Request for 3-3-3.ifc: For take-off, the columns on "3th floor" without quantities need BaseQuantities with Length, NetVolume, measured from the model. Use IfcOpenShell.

First a look at what the model holds.

```python
import ifcopenshell
import ifcopenshell.util.element
import ifcopenshell.util.unit

model = ifcopenshell.open("3-3-3.ifc")
print(model.schema)
for unit_type in ("LENGTHUNIT", "AREAUNIT", "VOLUMEUNIT"):
    print(unit_type, ifcopenshell.util.unit.calculate_unit_scale(model, unit_type))
storey = next(s for s in model.by_type("IfcBuildingStorey") if s.Name == "3th floor")
columns = [e for e in ifcopenshell.util.element.get_decomposition(storey) if e.is_a("IfcColumn")]
for e in sorted(columns, key=lambda e: e.id()):
    print(e.id(), e.is_a(), e.Name, list(ifcopenshell.util.element.get_psets(e, qtos_only=True)), sep=" | ")
```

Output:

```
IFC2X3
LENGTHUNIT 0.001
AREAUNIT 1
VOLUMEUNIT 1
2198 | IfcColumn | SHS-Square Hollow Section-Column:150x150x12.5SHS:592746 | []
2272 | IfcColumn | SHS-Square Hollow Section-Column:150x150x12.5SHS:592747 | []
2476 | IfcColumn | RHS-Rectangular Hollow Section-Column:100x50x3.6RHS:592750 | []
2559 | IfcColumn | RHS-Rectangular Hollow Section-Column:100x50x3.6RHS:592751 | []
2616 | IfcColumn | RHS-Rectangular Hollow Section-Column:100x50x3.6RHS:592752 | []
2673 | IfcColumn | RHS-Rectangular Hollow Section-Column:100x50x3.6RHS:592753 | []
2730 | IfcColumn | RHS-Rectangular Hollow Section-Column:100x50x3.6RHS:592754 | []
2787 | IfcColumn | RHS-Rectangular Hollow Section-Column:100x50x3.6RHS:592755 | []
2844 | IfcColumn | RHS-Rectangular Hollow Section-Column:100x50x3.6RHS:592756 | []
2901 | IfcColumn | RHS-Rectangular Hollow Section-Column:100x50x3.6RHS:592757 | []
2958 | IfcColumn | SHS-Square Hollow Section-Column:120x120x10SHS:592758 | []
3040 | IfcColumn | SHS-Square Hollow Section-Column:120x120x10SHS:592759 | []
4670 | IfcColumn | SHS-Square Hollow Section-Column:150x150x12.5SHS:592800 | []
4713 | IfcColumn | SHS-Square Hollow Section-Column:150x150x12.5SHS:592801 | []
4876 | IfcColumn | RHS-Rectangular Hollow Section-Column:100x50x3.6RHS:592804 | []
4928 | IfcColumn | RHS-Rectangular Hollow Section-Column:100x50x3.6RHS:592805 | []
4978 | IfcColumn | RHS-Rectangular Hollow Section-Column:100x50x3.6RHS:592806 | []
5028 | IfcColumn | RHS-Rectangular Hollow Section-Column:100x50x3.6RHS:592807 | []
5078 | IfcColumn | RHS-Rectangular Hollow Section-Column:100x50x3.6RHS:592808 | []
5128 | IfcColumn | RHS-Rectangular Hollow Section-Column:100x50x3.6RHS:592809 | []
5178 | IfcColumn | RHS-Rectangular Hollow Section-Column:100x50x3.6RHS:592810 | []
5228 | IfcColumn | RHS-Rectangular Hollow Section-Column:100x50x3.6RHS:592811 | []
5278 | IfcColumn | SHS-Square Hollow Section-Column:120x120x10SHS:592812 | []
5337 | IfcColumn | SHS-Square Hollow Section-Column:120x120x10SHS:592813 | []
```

```python
import ifcopenshell
import ifcopenshell.api.pset
import ifcopenshell.geom
import ifcopenshell.util.element
import ifcopenshell.util.shape
import ifcopenshell.util.unit

model = ifcopenshell.open("3-3-3.ifc")
unit_scale = ifcopenshell.util.unit.calculate_unit_scale(model)
volume_scale = ifcopenshell.util.unit.calculate_unit_scale(model, "VOLUMEUNIT")
settings = ifcopenshell.geom.settings()

storey = next(s for s in model.by_type("IfcBuildingStorey") if s.Name == "3th floor")
columns = [e for e in ifcopenshell.util.element.get_decomposition(storey) if e.is_a("IfcColumn")]

for e in sorted(columns, key=lambda e: e.id()):
    if ifcopenshell.util.element.get_psets(e, qtos_only=True, should_inherit=False):
        continue
    # Geometry comes back in metres, in the element's own axes.
    shape = ifcopenshell.geom.create_shape(settings, e)
    values = {
        "Length": ifcopenshell.util.shape.get_z(shape.geometry) / unit_scale,
        "NetVolume": ifcopenshell.util.shape.get_volume(shape.geometry) / volume_scale,
    }
    qto = ifcopenshell.api.pset.add_qto(model, product=e, name="BaseQuantities")
    ifcopenshell.api.pset.edit_qto(model, qto=qto, properties=values)
    print(e.id(), {k: round(v, 3) for k, v in values.items()})

model.write("3-3-3_v2.ifc")
```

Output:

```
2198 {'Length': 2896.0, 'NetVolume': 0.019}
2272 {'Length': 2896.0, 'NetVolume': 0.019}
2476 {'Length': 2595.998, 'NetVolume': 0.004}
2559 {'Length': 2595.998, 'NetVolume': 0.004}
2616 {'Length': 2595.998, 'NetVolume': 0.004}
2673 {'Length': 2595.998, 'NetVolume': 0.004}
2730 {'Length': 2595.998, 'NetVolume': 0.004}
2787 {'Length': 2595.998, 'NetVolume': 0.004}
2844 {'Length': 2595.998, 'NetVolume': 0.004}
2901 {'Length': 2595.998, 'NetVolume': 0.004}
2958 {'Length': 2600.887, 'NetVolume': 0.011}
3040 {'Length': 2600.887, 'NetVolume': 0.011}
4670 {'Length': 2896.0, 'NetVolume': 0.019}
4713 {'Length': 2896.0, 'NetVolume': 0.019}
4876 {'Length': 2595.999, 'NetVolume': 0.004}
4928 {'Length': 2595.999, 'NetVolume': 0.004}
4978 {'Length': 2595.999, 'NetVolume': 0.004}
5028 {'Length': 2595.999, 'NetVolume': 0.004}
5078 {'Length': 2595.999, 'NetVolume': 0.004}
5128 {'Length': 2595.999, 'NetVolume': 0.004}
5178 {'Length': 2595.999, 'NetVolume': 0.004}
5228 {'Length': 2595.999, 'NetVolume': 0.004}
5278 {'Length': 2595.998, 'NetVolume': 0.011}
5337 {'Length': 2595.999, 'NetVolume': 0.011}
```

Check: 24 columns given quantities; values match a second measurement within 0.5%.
